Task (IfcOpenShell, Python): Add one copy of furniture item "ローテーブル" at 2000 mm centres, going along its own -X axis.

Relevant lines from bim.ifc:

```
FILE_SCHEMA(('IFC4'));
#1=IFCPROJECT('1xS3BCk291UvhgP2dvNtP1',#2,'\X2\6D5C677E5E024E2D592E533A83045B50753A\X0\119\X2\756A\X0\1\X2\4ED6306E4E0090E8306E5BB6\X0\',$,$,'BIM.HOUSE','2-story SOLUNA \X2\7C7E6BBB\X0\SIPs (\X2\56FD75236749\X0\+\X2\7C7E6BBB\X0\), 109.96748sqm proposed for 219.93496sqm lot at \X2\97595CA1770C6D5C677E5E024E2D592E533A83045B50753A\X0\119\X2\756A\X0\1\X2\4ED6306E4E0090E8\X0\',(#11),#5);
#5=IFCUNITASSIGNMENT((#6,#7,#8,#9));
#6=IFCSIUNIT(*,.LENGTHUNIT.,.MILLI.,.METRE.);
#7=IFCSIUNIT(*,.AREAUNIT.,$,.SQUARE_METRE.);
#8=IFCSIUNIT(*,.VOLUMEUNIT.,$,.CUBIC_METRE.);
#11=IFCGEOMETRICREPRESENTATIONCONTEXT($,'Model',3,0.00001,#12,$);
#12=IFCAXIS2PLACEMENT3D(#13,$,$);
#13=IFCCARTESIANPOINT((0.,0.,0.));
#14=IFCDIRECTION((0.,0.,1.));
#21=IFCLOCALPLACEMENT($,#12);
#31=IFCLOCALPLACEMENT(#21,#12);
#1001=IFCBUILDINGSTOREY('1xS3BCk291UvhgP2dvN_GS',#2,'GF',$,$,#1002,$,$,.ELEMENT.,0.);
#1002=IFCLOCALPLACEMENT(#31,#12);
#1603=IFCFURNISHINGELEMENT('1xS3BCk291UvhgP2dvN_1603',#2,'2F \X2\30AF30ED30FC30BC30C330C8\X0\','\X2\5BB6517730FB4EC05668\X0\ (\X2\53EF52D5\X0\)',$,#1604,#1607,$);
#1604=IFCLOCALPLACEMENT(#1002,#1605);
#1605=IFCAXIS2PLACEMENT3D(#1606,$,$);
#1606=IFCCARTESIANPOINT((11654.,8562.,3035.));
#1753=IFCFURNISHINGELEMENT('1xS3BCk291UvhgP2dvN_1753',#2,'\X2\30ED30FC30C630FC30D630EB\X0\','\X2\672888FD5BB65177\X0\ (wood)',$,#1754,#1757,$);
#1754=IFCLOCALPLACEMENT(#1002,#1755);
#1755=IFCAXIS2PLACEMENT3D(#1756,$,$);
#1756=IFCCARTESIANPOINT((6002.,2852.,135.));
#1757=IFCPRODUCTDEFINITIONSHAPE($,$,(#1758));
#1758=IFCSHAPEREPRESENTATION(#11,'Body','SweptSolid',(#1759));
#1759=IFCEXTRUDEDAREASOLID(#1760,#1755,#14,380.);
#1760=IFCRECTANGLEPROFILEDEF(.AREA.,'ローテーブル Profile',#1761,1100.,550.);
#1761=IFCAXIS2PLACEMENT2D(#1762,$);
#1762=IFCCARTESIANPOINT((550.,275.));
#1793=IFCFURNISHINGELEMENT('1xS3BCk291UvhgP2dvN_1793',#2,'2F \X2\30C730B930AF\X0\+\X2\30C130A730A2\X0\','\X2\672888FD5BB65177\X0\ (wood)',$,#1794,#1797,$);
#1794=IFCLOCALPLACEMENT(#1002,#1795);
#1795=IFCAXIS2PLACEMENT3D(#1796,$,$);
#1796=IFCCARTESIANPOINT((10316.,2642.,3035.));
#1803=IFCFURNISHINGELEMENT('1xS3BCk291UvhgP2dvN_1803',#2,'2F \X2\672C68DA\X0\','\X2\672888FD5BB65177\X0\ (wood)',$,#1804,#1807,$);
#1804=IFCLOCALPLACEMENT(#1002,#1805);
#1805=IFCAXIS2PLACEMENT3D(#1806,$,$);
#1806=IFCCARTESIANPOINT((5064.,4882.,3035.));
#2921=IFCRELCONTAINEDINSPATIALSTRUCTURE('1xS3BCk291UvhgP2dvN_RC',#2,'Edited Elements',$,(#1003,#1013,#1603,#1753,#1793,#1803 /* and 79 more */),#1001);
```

```python
import ifcopenshell
import ifcopenshell.api.geometry
import ifcopenshell.api.root
import ifcopenshell.util.element
import ifcopenshell.util.placement
import ifcopenshell.util.unit

model = ifcopenshell.open("bim.ifc")
unit_scale = ifcopenshell.util.unit.calculate_unit_scale(model)


def reuse_history(source, copy):
    """copy_class also copies each property set's owner history, people and application; keep the originals."""
    for rel in copy.IsDefinedBy:
        if rel.is_a("IfcRelDefinesByProperties") and (history := rel.RelatingPropertyDefinition.OwnerHistory):
            rel.RelatingPropertyDefinition.OwnerHistory = source.OwnerHistory
            ifcopenshell.util.element.remove_deep2(model, history)


source = model.by_guid("1xS3BCk291UvhgP2dvN_1753")
base = ifcopenshell.util.placement.get_local_placement(source.ObjectPlacement)
step = -base[:3, 0] * 2 / unit_scale

for i in range(1, 2):
    copy = ifcopenshell.api.root.copy_class(model, product=source)
    copy.Representation = ifcopenshell.util.element.copy_deep(
        model, source.Representation, exclude=["IfcGeometricRepresentationContext", "IfcRepresentationMap"]
    )
    reuse_history(source, copy)
    matrix = base.copy()
    matrix[:3, 3] += i * step
    print("added at", matrix[:3, 3].round(3) + 0.0)
    ifcopenshell.api.geometry.edit_object_placement(model, product=copy, matrix=matrix, is_si=False)

model.write("bim-out.ifc")
```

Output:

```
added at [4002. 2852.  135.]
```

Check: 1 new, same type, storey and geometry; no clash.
